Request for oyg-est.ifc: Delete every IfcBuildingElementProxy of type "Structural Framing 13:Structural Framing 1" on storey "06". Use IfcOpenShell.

First a look at what the model holds.

```python
import ifcopenshell
import ifcopenshell.util.element

model = ifcopenshell.open("oyg-est.ifc")
print(model.schema)
storey = next(s for s in model.by_type("IfcBuildingStorey") if s.Name == "06")
proxies = [e for e in ifcopenshell.util.element.get_decomposition(storey) if e.is_a("IfcBuildingElementProxy")]
seen = {}
for e in proxies:
    element_type = ifcopenshell.util.element.get_type(e)
    name = element_type.Name if element_type not in (None, e) else None
    seen[name] = seen.get(name, 0) + 1
for name, count in sorted(seen.items(), key=str):
    print(count, "x", name)
```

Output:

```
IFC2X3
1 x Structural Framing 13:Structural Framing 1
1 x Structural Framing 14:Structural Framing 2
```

```python
import ifcopenshell
import ifcopenshell.api.root
import ifcopenshell.util.element

model = ifcopenshell.open("oyg-est.ifc")

storey = next(s for s in model.by_type("IfcBuildingStorey") if s.Name == "06")
proxies = [e for e in ifcopenshell.util.element.get_decomposition(storey) if e.is_a("IfcBuildingElementProxy")]
targets = [e for e in proxies if (t := ifcopenshell.util.element.get_type(e)) not in (None, e) and t.Name == "Structural Framing 13:Structural Framing 1"]

for e in targets:
    ifcopenshell.api.root.remove_product(model, product=e)
print(len(targets), "removed")

model.write("oyg-est_updated.ifc")
```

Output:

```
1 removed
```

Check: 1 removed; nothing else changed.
